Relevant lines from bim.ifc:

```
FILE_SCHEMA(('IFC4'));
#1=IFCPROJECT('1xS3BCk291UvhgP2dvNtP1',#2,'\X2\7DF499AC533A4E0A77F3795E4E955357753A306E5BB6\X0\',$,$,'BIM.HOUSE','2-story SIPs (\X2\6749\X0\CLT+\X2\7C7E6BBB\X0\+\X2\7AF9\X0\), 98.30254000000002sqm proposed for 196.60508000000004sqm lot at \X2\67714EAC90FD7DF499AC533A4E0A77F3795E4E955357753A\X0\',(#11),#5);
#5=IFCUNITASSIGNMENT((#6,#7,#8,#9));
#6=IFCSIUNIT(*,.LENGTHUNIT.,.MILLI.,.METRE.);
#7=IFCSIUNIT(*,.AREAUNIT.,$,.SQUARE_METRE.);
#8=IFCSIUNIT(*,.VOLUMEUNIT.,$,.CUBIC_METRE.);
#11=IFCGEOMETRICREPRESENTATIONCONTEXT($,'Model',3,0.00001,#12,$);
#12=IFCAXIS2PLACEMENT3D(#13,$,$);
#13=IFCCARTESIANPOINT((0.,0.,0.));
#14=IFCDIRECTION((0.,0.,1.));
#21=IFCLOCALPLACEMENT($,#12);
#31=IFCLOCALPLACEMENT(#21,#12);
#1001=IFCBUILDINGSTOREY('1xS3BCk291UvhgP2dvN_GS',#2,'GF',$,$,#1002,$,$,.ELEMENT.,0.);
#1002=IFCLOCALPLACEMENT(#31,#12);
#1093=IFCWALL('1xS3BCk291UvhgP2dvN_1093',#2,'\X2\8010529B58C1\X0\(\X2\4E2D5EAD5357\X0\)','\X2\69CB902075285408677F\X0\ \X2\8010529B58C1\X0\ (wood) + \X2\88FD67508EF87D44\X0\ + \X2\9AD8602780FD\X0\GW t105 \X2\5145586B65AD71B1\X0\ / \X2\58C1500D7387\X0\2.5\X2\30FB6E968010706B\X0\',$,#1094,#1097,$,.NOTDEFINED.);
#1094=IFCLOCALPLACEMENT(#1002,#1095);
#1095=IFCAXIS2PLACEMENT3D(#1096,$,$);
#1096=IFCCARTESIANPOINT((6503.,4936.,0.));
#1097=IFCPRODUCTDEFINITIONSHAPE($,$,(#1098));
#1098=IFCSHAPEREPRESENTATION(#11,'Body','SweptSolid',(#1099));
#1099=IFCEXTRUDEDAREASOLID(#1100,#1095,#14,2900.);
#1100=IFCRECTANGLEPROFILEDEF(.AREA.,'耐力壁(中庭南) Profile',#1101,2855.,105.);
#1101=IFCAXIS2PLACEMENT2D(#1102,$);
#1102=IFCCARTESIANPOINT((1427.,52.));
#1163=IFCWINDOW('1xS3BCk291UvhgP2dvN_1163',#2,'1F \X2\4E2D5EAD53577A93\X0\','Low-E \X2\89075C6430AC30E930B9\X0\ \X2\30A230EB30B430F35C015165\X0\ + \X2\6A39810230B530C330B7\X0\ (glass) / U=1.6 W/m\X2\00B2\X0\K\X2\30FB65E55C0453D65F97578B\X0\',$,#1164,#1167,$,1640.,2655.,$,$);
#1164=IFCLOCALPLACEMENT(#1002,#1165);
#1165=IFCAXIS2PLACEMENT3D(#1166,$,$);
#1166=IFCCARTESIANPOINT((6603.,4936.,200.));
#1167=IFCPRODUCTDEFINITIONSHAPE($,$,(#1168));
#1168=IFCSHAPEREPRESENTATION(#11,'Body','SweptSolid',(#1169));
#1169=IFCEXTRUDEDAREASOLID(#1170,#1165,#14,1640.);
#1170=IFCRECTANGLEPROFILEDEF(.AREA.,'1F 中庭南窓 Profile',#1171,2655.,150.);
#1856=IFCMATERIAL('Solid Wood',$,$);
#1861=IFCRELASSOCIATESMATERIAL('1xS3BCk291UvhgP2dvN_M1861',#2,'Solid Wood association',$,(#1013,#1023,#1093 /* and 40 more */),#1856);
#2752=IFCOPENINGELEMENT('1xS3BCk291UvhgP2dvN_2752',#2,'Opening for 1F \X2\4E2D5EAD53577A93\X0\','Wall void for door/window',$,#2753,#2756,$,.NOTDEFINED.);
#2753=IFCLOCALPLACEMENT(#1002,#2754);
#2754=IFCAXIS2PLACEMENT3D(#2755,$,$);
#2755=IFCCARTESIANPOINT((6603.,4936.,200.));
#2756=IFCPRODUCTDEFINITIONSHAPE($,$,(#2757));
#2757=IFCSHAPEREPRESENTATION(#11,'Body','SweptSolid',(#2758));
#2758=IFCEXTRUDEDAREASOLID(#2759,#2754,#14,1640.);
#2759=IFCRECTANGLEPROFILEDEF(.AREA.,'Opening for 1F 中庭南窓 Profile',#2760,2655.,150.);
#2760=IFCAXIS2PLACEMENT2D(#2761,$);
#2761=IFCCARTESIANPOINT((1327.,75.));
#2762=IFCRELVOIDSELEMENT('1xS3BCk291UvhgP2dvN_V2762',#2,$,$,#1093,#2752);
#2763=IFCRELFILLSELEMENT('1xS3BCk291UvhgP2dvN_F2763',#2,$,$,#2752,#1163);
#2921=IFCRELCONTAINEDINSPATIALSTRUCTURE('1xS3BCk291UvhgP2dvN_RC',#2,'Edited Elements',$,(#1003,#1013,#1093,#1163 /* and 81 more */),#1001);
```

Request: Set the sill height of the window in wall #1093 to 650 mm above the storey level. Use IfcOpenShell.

```python
import numpy as np
import ifcopenshell
import ifcopenshell.api.geometry
import ifcopenshell.geom
import ifcopenshell.util.element
import ifcopenshell.util.placement
import ifcopenshell.util.shape
import ifcopenshell.util.unit

model = ifcopenshell.open("bim.ifc")
unit_scale = ifcopenshell.util.unit.calculate_unit_scale(model)

window = model.by_guid("1xS3BCk291UvhgP2dvN_1163")
opening = window.FillsVoids[0].RelatingOpeningElement
storey = ifcopenshell.util.element.get_container(window, ifc_class="IfcBuildingStorey")
level = ifcopenshell.util.placement.get_local_placement(storey.ObjectPlacement)[2, 3]

# The opening's origin need not be at the sill, so measure its lowest point.
shape = ifcopenshell.geom.create_shape(ifcopenshell.geom.settings(), opening)
bottom = ifcopenshell.util.shape.get_shape_bottom_elevation(shape, shape.geometry) / unit_scale
dz = level + 0.65 / unit_scale - bottom

shift = np.array([0.0, 0.0, dz])
# The window is not placed relative to its opening, so move both.
for product in (opening, window):
    matrix = ifcopenshell.util.placement.get_local_placement(product.ObjectPlacement)
    matrix[:3, 3] += shift
    ifcopenshell.api.geometry.edit_object_placement(model, product=product, matrix=matrix, is_si=False)

print(f"moved by {dz * unit_scale:+.3f} m")

model.write("bim_edited.ifc")
```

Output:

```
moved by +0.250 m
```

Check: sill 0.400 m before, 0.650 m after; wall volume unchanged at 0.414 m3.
